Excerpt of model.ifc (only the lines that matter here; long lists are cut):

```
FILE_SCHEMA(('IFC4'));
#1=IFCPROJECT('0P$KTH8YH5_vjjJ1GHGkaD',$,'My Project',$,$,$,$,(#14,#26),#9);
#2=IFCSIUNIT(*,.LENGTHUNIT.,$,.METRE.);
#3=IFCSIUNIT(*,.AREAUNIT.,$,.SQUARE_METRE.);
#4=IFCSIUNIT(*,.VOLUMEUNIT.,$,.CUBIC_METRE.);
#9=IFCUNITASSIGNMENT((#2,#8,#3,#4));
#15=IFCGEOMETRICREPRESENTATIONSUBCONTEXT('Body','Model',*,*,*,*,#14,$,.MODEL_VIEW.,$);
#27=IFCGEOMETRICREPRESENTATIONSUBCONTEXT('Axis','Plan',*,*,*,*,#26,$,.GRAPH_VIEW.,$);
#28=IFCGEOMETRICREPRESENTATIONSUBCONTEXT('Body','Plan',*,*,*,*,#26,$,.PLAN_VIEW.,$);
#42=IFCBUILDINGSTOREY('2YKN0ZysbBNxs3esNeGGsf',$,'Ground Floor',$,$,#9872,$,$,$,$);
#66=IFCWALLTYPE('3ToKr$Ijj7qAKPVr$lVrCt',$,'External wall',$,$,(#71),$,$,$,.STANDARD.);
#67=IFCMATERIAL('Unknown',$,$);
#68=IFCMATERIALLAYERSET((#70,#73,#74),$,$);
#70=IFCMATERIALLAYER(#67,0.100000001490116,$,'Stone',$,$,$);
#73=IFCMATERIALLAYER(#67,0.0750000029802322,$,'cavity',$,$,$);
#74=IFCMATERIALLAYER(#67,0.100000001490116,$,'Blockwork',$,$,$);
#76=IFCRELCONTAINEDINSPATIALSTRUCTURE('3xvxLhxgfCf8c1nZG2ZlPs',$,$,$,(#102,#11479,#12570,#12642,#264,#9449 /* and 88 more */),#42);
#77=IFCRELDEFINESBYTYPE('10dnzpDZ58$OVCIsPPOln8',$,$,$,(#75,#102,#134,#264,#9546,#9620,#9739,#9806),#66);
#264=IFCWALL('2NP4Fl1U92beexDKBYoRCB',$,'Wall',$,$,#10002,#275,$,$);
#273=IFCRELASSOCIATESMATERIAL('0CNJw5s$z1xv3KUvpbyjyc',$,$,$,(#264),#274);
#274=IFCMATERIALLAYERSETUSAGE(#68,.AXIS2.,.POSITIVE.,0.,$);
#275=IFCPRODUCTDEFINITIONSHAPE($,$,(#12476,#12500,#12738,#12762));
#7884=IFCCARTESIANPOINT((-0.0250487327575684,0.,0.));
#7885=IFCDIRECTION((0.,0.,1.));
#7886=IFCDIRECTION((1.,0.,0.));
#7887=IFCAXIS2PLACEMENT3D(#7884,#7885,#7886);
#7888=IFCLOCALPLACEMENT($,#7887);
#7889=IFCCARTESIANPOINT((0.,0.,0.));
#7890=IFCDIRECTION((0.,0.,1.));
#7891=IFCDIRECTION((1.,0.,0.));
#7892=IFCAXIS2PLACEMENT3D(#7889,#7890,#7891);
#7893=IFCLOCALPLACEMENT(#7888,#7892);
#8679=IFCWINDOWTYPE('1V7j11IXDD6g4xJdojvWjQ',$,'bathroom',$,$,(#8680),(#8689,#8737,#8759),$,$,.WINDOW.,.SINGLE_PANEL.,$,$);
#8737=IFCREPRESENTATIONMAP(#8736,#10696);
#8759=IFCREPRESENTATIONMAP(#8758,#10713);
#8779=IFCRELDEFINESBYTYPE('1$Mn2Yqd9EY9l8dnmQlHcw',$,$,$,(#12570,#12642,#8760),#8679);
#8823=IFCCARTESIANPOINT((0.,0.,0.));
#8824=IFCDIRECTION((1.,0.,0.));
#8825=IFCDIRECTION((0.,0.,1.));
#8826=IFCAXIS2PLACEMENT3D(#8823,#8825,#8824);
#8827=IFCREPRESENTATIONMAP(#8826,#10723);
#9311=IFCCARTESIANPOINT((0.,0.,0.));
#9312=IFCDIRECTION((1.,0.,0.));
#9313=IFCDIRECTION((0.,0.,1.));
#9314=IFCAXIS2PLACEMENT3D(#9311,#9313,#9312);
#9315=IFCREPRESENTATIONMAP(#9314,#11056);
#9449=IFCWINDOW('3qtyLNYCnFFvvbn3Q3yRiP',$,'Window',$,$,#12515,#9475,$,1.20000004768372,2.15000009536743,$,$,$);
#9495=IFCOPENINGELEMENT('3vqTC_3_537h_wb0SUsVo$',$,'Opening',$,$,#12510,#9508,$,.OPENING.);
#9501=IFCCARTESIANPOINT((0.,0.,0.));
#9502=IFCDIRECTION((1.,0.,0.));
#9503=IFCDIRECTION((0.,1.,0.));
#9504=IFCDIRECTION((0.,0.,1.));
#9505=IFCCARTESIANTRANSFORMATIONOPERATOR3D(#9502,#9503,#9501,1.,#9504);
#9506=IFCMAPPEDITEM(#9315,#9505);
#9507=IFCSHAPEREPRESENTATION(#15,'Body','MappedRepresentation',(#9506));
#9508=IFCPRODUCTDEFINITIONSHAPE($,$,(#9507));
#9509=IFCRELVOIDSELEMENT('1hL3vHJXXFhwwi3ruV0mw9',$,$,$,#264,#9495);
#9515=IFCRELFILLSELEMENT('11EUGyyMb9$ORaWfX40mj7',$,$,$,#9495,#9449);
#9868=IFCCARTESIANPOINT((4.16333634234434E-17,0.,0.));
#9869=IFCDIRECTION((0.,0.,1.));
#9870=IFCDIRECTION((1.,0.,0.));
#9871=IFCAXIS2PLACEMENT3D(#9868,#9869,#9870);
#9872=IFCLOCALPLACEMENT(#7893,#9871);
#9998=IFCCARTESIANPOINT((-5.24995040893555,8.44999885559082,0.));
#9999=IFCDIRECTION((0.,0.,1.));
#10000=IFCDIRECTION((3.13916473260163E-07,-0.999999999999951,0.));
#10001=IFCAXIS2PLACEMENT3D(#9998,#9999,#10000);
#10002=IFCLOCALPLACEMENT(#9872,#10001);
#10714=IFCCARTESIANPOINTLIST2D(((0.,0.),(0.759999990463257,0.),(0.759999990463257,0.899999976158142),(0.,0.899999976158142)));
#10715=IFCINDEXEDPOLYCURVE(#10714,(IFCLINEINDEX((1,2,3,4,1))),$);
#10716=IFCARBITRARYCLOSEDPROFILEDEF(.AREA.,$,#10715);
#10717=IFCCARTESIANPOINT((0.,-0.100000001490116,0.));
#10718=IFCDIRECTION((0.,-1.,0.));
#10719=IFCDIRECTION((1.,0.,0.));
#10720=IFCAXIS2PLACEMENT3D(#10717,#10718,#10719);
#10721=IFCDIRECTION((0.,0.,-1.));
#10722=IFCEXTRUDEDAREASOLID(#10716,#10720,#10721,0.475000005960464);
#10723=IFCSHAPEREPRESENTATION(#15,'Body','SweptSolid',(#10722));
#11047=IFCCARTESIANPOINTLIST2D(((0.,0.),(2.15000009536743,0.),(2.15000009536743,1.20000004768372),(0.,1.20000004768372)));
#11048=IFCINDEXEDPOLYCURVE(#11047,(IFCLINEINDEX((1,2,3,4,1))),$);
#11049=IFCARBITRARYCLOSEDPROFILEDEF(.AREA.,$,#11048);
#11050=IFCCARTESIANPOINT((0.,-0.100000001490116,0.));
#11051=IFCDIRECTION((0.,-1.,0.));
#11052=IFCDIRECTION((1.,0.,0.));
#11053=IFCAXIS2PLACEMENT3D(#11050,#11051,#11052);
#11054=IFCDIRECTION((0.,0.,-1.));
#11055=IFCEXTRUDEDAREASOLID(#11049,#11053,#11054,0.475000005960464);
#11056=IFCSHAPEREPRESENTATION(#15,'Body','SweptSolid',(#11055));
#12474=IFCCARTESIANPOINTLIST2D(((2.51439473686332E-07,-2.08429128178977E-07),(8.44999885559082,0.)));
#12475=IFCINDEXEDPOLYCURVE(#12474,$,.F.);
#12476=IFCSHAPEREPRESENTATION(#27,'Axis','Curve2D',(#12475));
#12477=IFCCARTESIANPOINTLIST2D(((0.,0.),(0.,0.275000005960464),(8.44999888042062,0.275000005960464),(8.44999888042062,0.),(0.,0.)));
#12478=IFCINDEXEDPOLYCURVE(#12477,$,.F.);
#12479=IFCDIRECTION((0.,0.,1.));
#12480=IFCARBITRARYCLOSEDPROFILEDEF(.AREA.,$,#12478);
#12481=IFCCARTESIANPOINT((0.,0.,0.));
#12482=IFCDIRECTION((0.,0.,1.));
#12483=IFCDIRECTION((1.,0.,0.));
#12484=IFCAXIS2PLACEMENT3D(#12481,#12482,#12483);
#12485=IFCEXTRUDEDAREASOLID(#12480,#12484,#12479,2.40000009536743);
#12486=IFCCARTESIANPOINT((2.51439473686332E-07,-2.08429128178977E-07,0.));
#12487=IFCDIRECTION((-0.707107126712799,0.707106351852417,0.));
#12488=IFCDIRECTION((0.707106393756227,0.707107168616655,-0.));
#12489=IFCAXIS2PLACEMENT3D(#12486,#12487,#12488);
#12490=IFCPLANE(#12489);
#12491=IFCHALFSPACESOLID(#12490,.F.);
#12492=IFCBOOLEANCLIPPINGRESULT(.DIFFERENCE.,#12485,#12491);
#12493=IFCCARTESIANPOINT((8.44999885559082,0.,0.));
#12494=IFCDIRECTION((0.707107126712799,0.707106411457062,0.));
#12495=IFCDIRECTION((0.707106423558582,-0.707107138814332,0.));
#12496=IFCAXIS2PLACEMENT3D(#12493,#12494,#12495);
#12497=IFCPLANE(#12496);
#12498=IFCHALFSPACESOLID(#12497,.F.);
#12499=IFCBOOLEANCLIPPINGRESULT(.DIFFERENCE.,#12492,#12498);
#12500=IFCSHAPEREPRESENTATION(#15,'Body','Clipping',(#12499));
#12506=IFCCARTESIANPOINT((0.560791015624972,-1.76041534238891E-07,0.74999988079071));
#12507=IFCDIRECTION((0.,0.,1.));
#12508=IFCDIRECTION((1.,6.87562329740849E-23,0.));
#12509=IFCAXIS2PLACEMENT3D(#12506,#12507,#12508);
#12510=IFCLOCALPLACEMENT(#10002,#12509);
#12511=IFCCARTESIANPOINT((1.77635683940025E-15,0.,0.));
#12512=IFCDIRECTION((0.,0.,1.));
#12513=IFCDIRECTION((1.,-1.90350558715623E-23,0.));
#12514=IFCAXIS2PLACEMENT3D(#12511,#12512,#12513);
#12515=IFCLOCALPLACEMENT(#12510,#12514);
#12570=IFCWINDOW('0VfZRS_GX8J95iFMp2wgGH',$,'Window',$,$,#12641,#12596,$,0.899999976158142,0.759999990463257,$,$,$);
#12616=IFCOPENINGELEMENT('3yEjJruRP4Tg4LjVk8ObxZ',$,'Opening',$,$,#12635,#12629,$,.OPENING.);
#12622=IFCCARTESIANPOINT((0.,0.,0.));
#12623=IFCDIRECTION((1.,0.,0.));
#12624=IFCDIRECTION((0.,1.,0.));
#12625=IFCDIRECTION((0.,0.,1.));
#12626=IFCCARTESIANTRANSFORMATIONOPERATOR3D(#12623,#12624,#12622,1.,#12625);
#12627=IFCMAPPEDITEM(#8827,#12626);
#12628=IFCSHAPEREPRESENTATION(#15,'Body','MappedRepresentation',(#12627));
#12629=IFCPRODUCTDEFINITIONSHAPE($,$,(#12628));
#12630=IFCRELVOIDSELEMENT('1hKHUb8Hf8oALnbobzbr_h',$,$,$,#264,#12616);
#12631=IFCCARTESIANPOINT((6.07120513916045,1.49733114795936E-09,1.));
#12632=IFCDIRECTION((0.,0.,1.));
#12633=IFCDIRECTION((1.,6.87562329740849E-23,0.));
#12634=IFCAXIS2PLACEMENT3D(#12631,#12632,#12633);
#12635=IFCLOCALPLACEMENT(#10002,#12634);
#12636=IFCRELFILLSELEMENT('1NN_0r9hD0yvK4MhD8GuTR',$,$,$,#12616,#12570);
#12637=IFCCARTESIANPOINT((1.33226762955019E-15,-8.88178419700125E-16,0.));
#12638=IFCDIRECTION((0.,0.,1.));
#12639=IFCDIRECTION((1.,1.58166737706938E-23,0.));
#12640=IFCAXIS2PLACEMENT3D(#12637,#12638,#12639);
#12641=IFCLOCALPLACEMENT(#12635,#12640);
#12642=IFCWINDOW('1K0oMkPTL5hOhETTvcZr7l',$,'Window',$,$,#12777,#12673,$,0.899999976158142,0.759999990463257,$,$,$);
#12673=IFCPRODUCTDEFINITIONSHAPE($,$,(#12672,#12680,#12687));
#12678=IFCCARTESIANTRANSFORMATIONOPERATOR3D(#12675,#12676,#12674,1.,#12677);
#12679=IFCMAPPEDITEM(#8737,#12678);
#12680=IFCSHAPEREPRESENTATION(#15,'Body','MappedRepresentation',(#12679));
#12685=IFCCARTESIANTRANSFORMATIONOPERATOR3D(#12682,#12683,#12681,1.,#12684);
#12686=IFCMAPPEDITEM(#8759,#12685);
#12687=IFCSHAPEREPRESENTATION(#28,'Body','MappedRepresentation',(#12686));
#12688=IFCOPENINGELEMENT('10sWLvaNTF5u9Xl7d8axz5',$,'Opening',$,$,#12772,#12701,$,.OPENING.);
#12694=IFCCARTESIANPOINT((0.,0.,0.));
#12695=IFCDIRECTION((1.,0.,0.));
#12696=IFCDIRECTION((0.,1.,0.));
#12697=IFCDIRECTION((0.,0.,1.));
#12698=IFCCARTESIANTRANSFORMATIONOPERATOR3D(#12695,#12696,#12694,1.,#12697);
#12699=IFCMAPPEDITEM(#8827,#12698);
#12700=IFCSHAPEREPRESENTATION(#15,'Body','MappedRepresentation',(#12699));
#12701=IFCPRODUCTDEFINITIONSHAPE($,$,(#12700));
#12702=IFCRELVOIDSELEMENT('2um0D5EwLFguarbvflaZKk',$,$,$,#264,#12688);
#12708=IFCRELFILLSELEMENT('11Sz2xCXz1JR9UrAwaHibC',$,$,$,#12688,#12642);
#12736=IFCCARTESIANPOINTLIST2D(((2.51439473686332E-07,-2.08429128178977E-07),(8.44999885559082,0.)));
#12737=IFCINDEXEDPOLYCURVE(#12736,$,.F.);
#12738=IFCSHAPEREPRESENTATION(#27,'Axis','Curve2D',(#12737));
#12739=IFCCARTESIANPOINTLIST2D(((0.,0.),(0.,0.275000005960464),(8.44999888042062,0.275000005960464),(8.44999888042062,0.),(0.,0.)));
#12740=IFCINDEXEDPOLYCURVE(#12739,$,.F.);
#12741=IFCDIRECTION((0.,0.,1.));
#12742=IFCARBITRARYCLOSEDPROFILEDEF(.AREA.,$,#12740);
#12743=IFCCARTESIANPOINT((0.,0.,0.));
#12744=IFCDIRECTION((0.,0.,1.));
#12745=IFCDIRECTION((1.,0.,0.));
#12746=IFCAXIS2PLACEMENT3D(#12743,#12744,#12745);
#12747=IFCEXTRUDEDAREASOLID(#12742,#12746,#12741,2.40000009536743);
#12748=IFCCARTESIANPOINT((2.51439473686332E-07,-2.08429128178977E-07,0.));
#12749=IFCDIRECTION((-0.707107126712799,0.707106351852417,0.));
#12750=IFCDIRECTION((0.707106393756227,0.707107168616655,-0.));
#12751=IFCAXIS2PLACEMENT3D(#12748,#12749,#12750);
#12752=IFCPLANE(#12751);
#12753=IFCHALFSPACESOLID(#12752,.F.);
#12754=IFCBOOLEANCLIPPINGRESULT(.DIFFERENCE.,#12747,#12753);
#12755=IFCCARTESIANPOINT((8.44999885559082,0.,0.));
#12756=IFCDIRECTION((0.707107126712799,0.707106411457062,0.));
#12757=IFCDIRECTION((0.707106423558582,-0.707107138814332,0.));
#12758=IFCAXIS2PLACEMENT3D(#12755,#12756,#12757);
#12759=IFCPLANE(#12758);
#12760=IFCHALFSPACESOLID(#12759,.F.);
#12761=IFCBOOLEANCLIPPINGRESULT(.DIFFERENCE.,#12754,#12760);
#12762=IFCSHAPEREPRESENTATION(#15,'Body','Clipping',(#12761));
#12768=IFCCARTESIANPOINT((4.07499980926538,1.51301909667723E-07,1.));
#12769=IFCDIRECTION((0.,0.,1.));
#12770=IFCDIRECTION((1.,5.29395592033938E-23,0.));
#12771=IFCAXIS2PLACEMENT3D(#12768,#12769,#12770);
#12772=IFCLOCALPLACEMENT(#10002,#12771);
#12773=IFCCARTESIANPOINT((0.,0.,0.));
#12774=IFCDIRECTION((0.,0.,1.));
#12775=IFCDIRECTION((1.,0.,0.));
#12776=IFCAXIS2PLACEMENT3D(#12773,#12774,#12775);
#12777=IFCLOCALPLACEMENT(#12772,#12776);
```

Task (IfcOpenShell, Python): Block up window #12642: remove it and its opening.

```python
import ifcopenshell
import ifcopenshell.api.feature
import ifcopenshell.api.root
import ifcopenshell.geom
import ifcopenshell.util.shape

model = ifcopenshell.open("model.ifc")
settings = ifcopenshell.geom.settings()


def volume(element):
    """Net volume in cubic metres, openings subtracted."""
    shape = ifcopenshell.geom.create_shape(settings, element)
    return ifcopenshell.util.shape.get_volume(shape.geometry)


window = model.by_guid("1K0oMkPTL5hOhETTvcZr7l")
opening = window.FillsVoids[0].RelatingOpeningElement
wall = opening.VoidsElements[0].RelatingBuildingElement
before = volume(wall)

ifcopenshell.api.root.remove_product(model, product=window)
ifcopenshell.api.feature.remove_feature(model, feature=opening)

after = volume(wall)

print(f"wall volume {before:.3f} -> {after:.3f} m3")

model.write("model_rev.ifc")
```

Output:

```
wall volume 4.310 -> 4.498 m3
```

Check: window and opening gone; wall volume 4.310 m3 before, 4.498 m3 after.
